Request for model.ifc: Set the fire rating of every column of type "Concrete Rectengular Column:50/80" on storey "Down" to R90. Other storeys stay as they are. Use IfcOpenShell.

First a look at what the model holds.

```python
import ifcopenshell
import ifcopenshell.util.element

model = ifcopenshell.open("model.ifc")
print(model.schema)
storey = next(s for s in model.by_type("IfcBuildingStorey") if s.Name == "Down")
columns = [e for e in ifcopenshell.util.element.get_decomposition(storey) if e.is_a("IfcColumn")]
seen = {}
for e in columns:
    element_type = ifcopenshell.util.element.get_type(e)
    key = (element_type.Name if element_type != e and element_type else None, ifcopenshell.util.element.get_pset(e, "Pset_ColumnCommon", "FireRating"))
    seen[key] = seen.get(key, 0) + 1
for (name, value), count in sorted(seen.items(), key=str):
    print(count, "x", name, "|", value)
```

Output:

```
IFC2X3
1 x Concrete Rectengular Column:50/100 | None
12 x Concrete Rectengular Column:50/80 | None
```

```python
import ifcopenshell
import ifcopenshell.api.pset
import ifcopenshell.util.element

model = ifcopenshell.open("model.ifc")

storey = next(s for s in model.by_type("IfcBuildingStorey") if s.Name == "Down")
columns = [e for e in ifcopenshell.util.element.get_decomposition(storey) if e.is_a("IfcColumn")]

count = 0
for e in columns:
    element_type = ifcopenshell.util.element.get_type(e)
    if element_type in (None, e) or element_type.Name != "Concrete Rectengular Column:50/80":
        continue
    # add_pset returns the element's existing set when there is one.
    pset = ifcopenshell.api.pset.add_pset(model, product=e, name="Pset_ColumnCommon")
    ifcopenshell.api.pset.edit_pset(model, pset=pset, properties={"FireRating": "R90"})
    count += 1

print(count, "columns updated")

model.write("model_edited.ifc")
```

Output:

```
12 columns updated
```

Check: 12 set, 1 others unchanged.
